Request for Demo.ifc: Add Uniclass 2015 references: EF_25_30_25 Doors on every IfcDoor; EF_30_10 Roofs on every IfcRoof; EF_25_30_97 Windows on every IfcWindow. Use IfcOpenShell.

First a look at what the model holds.

```python
import ifcopenshell

model = ifcopenshell.open("Demo.ifc")
print(model.schema)
print("classifications:", [c.Name for c in model.by_type("IfcClassification")])
for ifc_class in ("IfcDoor", "IfcRoof", "IfcStair", "IfcWall", "IfcWindow"):
    print(ifc_class, len(model.by_type(ifc_class)))
```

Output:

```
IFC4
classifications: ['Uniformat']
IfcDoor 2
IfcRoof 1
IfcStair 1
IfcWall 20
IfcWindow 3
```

```python
import ifcopenshell
import ifcopenshell.api.classification

model = ifcopenshell.open("Demo.ifc")

system = ifcopenshell.api.classification.add_classification(model, classification="Uniclass 2015")

codes = {
    "IfcDoor": ("EF_25_30_25", "Doors"),
    "IfcRoof": ("EF_30_10", "Roofs"),
    "IfcWindow": ("EF_25_30_97", "Windows"),
}
for ifc_class, (code, name) in codes.items():
    products = model.by_type(ifc_class)
    ifcopenshell.api.classification.add_reference(
        model, products=products, classification=system, identification=code, name=name
    )
    print(code, len(products))

model.write("Demo_v2.ifc")
```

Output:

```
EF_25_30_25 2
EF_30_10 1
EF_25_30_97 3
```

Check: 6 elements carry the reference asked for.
